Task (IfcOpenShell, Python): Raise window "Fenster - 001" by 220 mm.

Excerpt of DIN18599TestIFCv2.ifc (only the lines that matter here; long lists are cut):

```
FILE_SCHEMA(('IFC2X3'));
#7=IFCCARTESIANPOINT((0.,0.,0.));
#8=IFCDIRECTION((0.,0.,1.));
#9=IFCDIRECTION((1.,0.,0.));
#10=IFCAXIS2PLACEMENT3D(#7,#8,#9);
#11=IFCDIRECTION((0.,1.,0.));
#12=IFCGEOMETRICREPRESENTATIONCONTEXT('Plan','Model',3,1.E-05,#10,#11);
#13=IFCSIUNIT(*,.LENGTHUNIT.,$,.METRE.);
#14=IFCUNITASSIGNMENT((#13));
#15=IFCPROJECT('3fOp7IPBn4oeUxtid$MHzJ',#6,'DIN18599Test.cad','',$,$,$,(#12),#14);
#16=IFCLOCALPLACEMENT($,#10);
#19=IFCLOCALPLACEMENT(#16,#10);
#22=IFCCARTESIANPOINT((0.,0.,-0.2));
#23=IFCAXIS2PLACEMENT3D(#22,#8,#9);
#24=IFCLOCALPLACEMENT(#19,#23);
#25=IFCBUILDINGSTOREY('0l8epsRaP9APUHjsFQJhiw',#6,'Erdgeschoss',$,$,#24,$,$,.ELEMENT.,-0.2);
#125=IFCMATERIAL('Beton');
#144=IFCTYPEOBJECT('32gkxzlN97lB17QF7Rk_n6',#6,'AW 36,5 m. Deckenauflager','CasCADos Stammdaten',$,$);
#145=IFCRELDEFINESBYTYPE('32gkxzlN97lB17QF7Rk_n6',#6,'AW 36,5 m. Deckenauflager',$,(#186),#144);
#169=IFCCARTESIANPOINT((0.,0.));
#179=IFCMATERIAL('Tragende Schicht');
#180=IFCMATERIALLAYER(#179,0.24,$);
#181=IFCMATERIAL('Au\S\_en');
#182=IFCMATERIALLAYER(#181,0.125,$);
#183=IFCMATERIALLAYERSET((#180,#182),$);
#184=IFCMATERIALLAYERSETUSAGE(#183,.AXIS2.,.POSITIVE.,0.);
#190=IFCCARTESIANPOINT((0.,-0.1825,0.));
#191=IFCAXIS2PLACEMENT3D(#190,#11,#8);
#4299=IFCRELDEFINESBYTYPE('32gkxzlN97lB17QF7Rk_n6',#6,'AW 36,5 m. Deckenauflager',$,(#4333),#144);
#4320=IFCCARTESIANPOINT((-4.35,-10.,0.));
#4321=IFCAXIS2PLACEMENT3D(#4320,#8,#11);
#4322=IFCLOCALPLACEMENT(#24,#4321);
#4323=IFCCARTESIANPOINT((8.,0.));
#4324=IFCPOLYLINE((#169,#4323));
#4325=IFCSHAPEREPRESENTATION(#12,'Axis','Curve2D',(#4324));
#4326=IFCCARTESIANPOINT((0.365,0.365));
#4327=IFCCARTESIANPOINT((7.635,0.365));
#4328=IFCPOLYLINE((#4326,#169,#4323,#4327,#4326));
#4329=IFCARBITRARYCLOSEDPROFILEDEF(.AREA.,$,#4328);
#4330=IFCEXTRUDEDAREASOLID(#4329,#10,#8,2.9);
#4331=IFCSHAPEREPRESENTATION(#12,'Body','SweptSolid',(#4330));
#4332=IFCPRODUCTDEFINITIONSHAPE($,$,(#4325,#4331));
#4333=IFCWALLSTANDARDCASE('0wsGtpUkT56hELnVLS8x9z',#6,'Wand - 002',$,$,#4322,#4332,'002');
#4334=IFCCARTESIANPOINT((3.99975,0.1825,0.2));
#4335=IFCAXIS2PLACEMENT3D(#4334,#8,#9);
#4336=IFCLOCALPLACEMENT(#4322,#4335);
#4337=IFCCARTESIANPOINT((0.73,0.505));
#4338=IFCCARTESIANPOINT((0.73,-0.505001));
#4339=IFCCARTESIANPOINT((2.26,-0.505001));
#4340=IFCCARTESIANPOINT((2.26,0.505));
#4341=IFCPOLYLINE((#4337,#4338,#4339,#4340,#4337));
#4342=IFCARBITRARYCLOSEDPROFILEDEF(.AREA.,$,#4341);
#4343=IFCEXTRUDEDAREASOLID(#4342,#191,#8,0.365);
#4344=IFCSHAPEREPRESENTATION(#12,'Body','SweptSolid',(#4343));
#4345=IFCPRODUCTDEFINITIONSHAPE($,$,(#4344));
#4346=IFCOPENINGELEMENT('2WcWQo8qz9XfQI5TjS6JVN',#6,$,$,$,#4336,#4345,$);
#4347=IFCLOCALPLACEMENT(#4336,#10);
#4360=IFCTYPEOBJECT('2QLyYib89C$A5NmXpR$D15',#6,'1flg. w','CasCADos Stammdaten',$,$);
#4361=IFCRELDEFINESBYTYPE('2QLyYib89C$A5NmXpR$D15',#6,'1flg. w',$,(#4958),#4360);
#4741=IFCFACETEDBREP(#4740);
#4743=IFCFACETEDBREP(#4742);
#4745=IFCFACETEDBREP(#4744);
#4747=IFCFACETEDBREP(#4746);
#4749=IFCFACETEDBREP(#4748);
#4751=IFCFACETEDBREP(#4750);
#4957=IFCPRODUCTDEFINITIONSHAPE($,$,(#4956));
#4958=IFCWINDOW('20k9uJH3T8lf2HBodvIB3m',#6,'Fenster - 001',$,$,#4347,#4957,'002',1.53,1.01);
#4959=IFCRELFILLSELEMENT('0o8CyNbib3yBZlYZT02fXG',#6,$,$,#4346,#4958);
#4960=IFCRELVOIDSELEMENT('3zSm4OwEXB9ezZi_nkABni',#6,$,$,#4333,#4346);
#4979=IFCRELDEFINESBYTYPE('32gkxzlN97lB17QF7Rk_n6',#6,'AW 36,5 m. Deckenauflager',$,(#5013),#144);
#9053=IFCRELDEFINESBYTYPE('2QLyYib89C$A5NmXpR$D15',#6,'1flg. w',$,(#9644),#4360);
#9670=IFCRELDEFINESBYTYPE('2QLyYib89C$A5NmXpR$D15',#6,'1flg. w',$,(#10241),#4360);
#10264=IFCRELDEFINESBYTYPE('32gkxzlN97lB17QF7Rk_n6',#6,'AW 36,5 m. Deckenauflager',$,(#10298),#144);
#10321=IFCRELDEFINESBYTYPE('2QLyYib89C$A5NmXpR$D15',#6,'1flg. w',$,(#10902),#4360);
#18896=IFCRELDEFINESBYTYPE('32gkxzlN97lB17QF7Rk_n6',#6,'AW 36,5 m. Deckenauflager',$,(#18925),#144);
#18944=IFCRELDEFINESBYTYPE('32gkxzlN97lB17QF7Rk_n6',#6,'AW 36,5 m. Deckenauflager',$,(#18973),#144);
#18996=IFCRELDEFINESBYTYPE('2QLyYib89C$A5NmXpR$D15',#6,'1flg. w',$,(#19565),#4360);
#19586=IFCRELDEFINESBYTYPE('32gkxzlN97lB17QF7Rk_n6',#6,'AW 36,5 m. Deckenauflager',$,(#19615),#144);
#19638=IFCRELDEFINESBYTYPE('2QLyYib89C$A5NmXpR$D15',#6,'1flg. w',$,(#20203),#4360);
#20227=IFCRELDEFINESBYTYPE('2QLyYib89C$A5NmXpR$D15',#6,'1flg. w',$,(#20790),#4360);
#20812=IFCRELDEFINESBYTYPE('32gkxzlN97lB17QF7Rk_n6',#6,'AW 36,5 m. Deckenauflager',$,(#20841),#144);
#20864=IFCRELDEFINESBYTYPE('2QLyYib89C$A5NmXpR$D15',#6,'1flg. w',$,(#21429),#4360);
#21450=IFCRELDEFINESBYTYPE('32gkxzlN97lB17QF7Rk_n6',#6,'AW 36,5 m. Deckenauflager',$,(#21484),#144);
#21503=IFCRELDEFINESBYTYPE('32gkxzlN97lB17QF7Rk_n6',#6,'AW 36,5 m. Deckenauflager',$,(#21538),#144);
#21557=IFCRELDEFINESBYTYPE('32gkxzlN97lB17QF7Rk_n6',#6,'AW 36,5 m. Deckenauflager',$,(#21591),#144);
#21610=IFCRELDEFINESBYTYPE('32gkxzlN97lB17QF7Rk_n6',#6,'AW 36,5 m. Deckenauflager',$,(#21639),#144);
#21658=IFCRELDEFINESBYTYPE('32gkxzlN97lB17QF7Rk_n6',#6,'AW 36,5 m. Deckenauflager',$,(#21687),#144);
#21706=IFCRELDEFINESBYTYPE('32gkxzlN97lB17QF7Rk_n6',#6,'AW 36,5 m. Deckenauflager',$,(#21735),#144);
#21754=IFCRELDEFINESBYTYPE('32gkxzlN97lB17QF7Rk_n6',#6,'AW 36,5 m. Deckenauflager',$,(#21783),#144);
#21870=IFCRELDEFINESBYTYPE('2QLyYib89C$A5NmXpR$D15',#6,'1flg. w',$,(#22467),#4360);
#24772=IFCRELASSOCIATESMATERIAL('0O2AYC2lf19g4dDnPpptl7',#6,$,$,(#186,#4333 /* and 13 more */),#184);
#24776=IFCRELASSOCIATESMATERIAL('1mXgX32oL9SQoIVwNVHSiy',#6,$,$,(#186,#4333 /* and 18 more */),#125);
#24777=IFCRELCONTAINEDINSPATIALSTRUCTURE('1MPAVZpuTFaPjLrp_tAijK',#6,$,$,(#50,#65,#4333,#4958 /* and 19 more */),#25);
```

```python
import numpy as np
import ifcopenshell
import ifcopenshell.api.geometry
import ifcopenshell.util.placement
import ifcopenshell.util.unit

model = ifcopenshell.open("DIN18599TestIFCv2.ifc")
unit_scale = ifcopenshell.util.unit.calculate_unit_scale(model)

window = model.by_id(4958)
opening = window.FillsVoids[0].RelatingOpeningElement
dz = 0.22 / unit_scale

shift = np.array([0.0, 0.0, dz])
# The window is placed relative to its opening, so it follows when the opening moves.
matrix = ifcopenshell.util.placement.get_local_placement(opening.ObjectPlacement)
matrix[:3, 3] += shift
ifcopenshell.api.geometry.edit_object_placement(
    model, product=opening, matrix=matrix, is_si=False, should_transform_children=True
)

print(f"moved by {dz * unit_scale:+.3f} m")

model.write("DIN18599TestIFCv2_updated.ifc")
```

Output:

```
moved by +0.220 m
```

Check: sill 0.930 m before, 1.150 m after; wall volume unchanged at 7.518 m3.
